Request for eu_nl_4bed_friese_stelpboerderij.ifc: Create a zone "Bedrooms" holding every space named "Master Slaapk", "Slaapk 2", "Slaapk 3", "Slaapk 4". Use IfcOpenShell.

First a look at what the model holds.

```python
import ifcopenshell

model = ifcopenshell.open("eu_nl_4bed_friese_stelpboerderij.ifc")
print(model.schema)
seen = {}
for space in model.by_type("IfcSpace"):
    seen[space.LongName] = seen.get(space.LongName, 0) + 1
for name, count in sorted(seen.items(), key=str):
    print(count, "x", name)
print("zones:", [z.Name for z in model.by_type("IfcZone")][:20])
```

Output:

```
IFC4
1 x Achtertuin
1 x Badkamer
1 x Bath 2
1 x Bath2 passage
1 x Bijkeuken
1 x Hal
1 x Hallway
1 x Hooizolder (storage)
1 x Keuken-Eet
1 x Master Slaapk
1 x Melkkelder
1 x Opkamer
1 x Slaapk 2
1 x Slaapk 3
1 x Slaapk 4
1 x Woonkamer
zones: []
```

```python
import ifcopenshell
import ifcopenshell.api.group
import ifcopenshell.api.root

model = ifcopenshell.open("eu_nl_4bed_friese_stelpboerderij.ifc")

names = {"Master Slaapk", "Slaapk 2", "Slaapk 3", "Slaapk 4"}
spaces = [s for s in model.by_type("IfcSpace") if s.LongName in names]

zone = ifcopenshell.api.root.create_entity(model, ifc_class="IfcZone", name="Bedrooms")
ifcopenshell.api.group.assign_group(model, products=spaces, group=zone)
print(len(spaces), "spaces in", zone.Name)

model.write("eu_nl_4bed_friese_stelpboerderij_updated.ifc")
```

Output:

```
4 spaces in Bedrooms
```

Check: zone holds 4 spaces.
